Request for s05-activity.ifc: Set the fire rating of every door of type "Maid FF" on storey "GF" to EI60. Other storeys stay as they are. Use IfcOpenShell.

First a look at what the model holds.

```python
import ifcopenshell
import ifcopenshell.util.element

model = ifcopenshell.open("s05-activity.ifc")
print(model.schema)
storey = next(s for s in model.by_type("IfcBuildingStorey") if s.Name == "GF")
doors = [e for e in ifcopenshell.util.element.get_decomposition(storey) if e.is_a("IfcDoor")]
seen = {}
for e in doors:
    element_type = ifcopenshell.util.element.get_type(e)
    key = (element_type.Name if element_type != e and element_type else None, ifcopenshell.util.element.get_pset(e, "Pset_DoorCommon", "FireRating"))
    seen[key] = seen.get(key, 0) + 1
for (name, value), count in sorted(seen.items(), key=str):
    print(count, "x", name, "|", value)
```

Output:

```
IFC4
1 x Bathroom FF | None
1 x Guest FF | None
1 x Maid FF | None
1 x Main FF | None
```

```python
import ifcopenshell
import ifcopenshell.api.pset
import ifcopenshell.util.element

model = ifcopenshell.open("s05-activity.ifc")

storey = next(s for s in model.by_type("IfcBuildingStorey") if s.Name == "GF")
doors = [e for e in ifcopenshell.util.element.get_decomposition(storey) if e.is_a("IfcDoor")]

count = 0
for e in doors:
    element_type = ifcopenshell.util.element.get_type(e)
    if element_type in (None, e) or element_type.Name != "Maid FF":
        continue
    # add_pset returns the element's existing set when there is one.
    pset = ifcopenshell.api.pset.add_pset(model, product=e, name="Pset_DoorCommon")
    ifcopenshell.api.pset.edit_pset(model, pset=pset, properties={"FireRating": "EI60"})
    count += 1

print(count, "doors updated")

model.write("s05-activity-out.ifc")
```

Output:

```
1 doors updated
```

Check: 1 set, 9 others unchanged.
